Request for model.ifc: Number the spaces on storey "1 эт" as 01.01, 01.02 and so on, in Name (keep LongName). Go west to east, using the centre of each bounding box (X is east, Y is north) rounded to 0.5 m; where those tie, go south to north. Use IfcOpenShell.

First a look at what the model holds.

```python
import ifcopenshell
import ifcopenshell.util.element
import ifcopenshell.util.placement

model = ifcopenshell.open("model.ifc")
print(model.schema)
storey = next(s for s in model.by_type("IfcBuildingStorey") if s.Name == "1 эт")
spaces = [e for e in ifcopenshell.util.element.get_decomposition(storey) if e.is_a("IfcSpace")]
for e in sorted(spaces, key=lambda e: e.id()):
    origin = ifcopenshell.util.placement.get_local_placement(e.ObjectPlacement)[:3, 3]
    print(e.id(), e.Name, e.LongName, origin.round(2) + 0.0, sep=" | ")
```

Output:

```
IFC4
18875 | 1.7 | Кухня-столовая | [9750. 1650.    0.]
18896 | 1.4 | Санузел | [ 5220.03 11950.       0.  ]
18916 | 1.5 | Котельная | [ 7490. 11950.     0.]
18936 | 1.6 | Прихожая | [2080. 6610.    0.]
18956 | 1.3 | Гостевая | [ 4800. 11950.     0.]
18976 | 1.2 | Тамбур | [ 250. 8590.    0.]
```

```python
import ifcopenshell
import ifcopenshell.geom
import ifcopenshell.util.element
import ifcopenshell.util.shape

model = ifcopenshell.open("model.ifc")
settings = ifcopenshell.geom.settings()
settings.set("use-world-coords", True)


def centre(element):
    shape = ifcopenshell.geom.create_shape(settings, element)
    return ifcopenshell.util.shape.get_bbox_centroid(shape.geometry)


storey = next(s for s in model.by_type("IfcBuildingStorey") if s.Name == "1 эт")
spaces = [e for e in ifcopenshell.util.element.get_decomposition(storey) if e.is_a("IfcSpace")]

# Insertion points can sit at a corner or the storey origin, so sort by the geometry (in metres).
centres = {e: centre(e) for e in spaces}
spaces.sort(key=lambda e: (round(centres[e][0] / 0.5), centres[e][1]))

for i, e in enumerate(spaces, start=1):
    number = f"01.{i:02d}"
    e.Name = number
    print(e.id(), number)

model.write("model_v2.ifc")
```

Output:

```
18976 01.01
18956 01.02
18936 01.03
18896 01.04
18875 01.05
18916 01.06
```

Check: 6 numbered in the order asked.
